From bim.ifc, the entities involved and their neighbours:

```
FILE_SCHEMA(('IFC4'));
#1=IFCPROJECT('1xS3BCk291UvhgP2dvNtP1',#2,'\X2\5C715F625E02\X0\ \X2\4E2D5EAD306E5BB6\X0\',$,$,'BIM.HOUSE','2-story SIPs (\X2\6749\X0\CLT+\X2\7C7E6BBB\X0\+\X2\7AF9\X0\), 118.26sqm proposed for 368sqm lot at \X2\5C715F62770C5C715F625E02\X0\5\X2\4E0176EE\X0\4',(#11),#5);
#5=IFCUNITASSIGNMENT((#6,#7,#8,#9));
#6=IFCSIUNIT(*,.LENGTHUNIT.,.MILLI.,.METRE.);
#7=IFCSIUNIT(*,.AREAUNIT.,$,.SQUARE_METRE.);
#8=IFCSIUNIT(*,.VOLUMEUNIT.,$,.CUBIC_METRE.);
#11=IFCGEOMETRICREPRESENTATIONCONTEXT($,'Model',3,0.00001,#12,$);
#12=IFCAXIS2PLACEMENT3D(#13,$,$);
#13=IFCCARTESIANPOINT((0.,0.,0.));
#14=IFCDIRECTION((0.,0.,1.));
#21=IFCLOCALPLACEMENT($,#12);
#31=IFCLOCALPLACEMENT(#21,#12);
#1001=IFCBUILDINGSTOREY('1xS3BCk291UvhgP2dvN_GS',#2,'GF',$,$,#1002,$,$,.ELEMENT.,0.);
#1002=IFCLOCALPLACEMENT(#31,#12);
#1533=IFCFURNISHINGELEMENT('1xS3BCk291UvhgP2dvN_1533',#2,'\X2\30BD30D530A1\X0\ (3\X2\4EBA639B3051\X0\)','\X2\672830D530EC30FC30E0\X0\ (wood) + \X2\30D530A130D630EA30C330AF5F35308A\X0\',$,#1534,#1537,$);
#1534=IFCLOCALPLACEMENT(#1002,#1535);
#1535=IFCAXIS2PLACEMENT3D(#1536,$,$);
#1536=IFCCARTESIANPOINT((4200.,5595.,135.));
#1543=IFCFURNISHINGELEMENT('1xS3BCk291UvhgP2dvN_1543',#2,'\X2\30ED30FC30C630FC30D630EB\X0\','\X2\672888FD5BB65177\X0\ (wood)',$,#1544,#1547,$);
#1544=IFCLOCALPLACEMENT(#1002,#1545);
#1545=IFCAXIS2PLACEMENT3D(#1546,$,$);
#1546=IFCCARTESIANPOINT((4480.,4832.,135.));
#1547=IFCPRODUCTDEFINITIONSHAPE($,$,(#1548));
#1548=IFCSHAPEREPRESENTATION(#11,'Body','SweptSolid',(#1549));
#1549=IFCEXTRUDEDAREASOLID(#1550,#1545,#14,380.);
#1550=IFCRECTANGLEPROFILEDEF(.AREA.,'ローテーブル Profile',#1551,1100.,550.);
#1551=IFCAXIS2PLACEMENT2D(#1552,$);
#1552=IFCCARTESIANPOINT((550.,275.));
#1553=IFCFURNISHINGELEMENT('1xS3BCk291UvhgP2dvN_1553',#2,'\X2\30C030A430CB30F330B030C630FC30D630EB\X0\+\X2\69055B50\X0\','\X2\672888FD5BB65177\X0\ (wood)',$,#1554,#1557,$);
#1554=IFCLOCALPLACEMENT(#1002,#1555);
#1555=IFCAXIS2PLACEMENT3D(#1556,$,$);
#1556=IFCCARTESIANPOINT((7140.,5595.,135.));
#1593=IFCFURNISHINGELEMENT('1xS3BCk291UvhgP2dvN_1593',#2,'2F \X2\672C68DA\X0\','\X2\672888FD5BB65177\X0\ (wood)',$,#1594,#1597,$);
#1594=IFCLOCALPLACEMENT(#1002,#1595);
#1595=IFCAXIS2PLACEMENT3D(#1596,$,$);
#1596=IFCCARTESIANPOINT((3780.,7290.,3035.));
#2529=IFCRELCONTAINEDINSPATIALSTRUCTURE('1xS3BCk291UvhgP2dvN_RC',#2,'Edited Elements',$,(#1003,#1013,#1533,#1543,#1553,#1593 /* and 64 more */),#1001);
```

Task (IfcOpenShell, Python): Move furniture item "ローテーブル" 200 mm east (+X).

```python
import ifcopenshell
import ifcopenshell.api.geometry
import ifcopenshell.util.placement
import ifcopenshell.util.unit

model = ifcopenshell.open("bim.ifc")
unit_scale = ifcopenshell.util.unit.calculate_unit_scale(model)

item = model.by_guid("1xS3BCk291UvhgP2dvN_1543")
matrix = ifcopenshell.util.placement.get_local_placement(item.ObjectPlacement)
matrix[0, 3] += 0.2 / unit_scale
ifcopenshell.api.geometry.edit_object_placement(model, product=item, matrix=matrix, is_si=False)

print(ifcopenshell.util.placement.get_local_placement(item.ObjectPlacement).round(3) + 0.0)

model.write("bim-out.ifc")
```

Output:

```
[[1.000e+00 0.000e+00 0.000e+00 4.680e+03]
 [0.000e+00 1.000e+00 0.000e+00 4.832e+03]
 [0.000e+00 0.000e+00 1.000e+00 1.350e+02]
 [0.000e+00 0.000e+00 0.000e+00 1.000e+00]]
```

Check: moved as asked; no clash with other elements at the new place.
